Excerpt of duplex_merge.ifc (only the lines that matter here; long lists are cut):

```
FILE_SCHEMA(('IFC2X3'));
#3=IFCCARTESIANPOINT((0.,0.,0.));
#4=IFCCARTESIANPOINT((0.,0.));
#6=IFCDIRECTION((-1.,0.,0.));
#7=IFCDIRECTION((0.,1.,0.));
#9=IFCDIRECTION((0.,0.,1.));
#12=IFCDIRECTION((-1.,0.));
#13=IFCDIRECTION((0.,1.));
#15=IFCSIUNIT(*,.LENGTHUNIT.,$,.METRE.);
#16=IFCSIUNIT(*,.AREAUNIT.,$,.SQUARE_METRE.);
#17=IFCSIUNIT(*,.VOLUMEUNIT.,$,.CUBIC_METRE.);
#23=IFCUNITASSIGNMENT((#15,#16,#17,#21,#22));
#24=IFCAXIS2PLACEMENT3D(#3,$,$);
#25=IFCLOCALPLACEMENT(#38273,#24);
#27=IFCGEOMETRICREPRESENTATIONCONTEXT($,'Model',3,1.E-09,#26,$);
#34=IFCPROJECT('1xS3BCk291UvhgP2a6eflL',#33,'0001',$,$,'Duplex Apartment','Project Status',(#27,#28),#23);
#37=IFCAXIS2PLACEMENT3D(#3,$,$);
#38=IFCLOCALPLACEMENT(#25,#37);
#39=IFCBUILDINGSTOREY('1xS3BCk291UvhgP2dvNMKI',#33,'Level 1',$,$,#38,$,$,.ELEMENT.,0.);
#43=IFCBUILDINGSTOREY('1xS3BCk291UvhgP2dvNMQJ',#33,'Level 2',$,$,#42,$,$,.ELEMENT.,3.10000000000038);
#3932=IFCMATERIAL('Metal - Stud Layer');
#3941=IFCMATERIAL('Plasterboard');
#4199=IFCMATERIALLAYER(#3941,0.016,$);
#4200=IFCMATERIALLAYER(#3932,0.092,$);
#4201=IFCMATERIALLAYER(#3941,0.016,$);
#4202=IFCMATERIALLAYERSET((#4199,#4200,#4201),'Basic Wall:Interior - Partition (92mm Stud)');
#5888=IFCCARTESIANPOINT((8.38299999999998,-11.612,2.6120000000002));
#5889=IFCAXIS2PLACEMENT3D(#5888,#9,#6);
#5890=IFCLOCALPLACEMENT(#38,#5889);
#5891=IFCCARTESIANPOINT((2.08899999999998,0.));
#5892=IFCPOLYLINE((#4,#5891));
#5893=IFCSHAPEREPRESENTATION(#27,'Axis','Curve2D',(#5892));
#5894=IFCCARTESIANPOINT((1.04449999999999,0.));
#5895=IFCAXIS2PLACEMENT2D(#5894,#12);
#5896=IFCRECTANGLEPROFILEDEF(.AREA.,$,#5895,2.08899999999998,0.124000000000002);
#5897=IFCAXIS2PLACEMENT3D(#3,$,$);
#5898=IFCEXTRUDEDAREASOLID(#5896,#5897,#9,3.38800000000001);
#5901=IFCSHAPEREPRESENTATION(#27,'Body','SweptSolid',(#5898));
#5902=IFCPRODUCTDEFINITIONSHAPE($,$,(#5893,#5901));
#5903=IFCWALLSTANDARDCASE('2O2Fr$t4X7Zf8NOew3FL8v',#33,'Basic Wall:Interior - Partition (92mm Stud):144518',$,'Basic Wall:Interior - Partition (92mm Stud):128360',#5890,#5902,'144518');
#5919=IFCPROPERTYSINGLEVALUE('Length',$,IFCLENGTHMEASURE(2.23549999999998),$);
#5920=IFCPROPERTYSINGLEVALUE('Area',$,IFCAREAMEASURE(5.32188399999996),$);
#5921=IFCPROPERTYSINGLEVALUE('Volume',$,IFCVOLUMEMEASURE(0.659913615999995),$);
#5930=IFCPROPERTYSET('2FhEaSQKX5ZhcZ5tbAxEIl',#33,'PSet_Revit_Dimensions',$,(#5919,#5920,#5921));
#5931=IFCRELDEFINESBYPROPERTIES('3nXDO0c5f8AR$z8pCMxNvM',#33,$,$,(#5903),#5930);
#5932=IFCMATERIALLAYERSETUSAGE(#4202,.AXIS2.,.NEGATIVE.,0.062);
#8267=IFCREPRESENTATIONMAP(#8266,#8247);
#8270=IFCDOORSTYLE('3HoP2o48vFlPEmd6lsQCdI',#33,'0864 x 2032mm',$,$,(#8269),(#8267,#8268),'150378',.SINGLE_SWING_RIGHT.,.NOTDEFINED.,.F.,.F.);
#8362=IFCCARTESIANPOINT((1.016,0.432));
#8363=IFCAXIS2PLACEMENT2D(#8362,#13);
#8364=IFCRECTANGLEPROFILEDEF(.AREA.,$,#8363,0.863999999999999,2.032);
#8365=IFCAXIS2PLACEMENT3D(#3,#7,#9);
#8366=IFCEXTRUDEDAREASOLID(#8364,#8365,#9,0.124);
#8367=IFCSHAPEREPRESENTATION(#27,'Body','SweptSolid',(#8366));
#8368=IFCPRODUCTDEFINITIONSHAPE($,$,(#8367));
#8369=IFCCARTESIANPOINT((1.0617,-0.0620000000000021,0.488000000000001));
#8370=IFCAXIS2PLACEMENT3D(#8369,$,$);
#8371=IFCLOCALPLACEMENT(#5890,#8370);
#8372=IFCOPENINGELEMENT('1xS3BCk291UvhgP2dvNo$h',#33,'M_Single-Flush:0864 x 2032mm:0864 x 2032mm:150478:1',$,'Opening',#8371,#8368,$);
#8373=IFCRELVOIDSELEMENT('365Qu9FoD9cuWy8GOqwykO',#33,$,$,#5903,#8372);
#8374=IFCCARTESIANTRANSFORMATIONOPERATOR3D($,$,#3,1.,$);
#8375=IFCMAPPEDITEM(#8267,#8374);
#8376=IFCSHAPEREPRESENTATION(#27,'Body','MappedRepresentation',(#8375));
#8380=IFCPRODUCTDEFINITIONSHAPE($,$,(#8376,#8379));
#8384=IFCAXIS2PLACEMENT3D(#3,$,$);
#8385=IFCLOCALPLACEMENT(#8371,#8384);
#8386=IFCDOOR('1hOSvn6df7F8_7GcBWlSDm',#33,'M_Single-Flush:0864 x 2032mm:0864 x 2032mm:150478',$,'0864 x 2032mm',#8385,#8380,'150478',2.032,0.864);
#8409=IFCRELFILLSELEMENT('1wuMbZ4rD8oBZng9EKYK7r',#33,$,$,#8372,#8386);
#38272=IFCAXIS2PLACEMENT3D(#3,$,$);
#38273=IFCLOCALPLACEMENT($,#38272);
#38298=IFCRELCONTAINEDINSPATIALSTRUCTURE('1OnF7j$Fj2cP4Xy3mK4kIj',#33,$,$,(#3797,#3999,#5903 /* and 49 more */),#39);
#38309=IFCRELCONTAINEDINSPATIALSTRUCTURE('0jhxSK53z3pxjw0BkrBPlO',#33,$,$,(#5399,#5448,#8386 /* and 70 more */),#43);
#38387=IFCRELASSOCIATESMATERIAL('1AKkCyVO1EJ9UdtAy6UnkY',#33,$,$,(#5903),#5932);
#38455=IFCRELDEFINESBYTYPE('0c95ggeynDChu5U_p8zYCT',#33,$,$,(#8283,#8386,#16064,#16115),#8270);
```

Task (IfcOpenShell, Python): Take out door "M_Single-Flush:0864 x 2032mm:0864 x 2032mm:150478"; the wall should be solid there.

```python
import ifcopenshell
import ifcopenshell.api.feature
import ifcopenshell.api.pset
import ifcopenshell.api.root
import ifcopenshell.geom
import ifcopenshell.util.element
import ifcopenshell.util.shape
import ifcopenshell.util.unit

model = ifcopenshell.open("duplex_merge.ifc")
area_scale = ifcopenshell.util.unit.calculate_unit_scale(model, "AREAUNIT")
volume_scale = ifcopenshell.util.unit.calculate_unit_scale(model, "VOLUMEUNIT")
settings = ifcopenshell.geom.settings()


def volume(element):
    """Net volume in cubic metres, openings subtracted."""
    shape = ifcopenshell.geom.create_shape(settings, element)
    return ifcopenshell.util.shape.get_volume(shape.geometry)


door = model.by_id(8386)
opening = door.FillsVoids[0].RelatingOpeningElement
wall = opening.VoidsElements[0].RelatingBuildingElement
before = volume(wall)

ifcopenshell.api.root.remove_product(model, product=door)
ifcopenshell.api.feature.remove_feature(model, feature=opening)

after = volume(wall)
thickness = 0.124  # wall thickness in metres

# Update the wall's stored quantities.
pset = model.by_id(ifcopenshell.util.element.get_pset(wall, "PSet_Revit_Dimensions", should_inherit=False)["id"])
ifcopenshell.api.pset.edit_pset(model, pset=pset, properties={
    "Area": model.create_entity("IfcAreaMeasure", after / thickness / area_scale),
    "Volume": model.create_entity("IfcVolumeMeasure", after / volume_scale),
})

print(f"wall volume {before:.3f} -> {after:.3f} m3")

model.write("duplex_merge_updated.ifc")
```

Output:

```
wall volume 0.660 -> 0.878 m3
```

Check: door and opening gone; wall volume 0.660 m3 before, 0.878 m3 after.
